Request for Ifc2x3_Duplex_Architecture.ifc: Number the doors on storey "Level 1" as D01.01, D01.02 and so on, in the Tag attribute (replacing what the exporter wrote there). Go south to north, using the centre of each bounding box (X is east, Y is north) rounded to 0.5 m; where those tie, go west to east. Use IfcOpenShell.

First a look at what the model holds.

```python
import ifcopenshell
import ifcopenshell.util.element
import ifcopenshell.util.placement

model = ifcopenshell.open("Ifc2x3_Duplex_Architecture.ifc")
print(model.schema)
storey = next(s for s in model.by_type("IfcBuildingStorey") if s.Name == "Level 1")
doors = [e for e in ifcopenshell.util.element.get_decomposition(storey) if e.is_a("IfcDoor")]
for e in sorted(doors, key=lambda e: e.id()):
    origin = ifcopenshell.util.placement.get_local_placement(e.ObjectPlacement)[:3, 3]
    print(e.id(), e.Tag, e.Name, origin.round(2) + 0.0, sep=" | ")
```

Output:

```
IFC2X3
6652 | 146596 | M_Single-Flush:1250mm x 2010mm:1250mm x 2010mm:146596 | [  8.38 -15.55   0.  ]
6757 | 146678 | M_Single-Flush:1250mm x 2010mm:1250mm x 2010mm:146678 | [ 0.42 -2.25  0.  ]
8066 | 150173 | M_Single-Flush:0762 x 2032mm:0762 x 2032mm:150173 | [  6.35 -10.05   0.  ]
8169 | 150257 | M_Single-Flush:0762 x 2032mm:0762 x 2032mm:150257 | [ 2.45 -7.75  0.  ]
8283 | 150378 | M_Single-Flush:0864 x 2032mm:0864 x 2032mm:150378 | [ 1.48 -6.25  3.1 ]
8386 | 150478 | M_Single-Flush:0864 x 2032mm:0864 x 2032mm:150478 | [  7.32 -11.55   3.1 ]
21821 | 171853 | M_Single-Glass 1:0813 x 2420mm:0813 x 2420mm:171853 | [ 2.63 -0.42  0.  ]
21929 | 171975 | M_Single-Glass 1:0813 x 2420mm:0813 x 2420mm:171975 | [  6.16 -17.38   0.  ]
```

```python
import ifcopenshell
import ifcopenshell.geom
import ifcopenshell.util.element
import ifcopenshell.util.shape

model = ifcopenshell.open("Ifc2x3_Duplex_Architecture.ifc")
settings = ifcopenshell.geom.settings()
settings.set("use-world-coords", True)


def centre(element):
    shape = ifcopenshell.geom.create_shape(settings, element)
    return ifcopenshell.util.shape.get_bbox_centroid(shape.geometry)


storey = next(s for s in model.by_type("IfcBuildingStorey") if s.Name == "Level 1")
doors = [e for e in ifcopenshell.util.element.get_decomposition(storey) if e.is_a("IfcDoor")]

# Insertion points can sit at a corner or the storey origin, so sort by the geometry (in metres).
centres = {e: centre(e) for e in doors}
doors.sort(key=lambda e: (round(centres[e][1] / 0.5), centres[e][0]))

for i, e in enumerate(doors, start=1):
    number = f"D01.{i:02d}"
    e.Tag = number
    print(e.id(), number)

model.write("Ifc2x3_Duplex_Architecture_v2.ifc")
```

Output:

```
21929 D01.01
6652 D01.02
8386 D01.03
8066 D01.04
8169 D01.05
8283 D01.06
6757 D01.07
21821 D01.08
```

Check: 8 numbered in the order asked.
